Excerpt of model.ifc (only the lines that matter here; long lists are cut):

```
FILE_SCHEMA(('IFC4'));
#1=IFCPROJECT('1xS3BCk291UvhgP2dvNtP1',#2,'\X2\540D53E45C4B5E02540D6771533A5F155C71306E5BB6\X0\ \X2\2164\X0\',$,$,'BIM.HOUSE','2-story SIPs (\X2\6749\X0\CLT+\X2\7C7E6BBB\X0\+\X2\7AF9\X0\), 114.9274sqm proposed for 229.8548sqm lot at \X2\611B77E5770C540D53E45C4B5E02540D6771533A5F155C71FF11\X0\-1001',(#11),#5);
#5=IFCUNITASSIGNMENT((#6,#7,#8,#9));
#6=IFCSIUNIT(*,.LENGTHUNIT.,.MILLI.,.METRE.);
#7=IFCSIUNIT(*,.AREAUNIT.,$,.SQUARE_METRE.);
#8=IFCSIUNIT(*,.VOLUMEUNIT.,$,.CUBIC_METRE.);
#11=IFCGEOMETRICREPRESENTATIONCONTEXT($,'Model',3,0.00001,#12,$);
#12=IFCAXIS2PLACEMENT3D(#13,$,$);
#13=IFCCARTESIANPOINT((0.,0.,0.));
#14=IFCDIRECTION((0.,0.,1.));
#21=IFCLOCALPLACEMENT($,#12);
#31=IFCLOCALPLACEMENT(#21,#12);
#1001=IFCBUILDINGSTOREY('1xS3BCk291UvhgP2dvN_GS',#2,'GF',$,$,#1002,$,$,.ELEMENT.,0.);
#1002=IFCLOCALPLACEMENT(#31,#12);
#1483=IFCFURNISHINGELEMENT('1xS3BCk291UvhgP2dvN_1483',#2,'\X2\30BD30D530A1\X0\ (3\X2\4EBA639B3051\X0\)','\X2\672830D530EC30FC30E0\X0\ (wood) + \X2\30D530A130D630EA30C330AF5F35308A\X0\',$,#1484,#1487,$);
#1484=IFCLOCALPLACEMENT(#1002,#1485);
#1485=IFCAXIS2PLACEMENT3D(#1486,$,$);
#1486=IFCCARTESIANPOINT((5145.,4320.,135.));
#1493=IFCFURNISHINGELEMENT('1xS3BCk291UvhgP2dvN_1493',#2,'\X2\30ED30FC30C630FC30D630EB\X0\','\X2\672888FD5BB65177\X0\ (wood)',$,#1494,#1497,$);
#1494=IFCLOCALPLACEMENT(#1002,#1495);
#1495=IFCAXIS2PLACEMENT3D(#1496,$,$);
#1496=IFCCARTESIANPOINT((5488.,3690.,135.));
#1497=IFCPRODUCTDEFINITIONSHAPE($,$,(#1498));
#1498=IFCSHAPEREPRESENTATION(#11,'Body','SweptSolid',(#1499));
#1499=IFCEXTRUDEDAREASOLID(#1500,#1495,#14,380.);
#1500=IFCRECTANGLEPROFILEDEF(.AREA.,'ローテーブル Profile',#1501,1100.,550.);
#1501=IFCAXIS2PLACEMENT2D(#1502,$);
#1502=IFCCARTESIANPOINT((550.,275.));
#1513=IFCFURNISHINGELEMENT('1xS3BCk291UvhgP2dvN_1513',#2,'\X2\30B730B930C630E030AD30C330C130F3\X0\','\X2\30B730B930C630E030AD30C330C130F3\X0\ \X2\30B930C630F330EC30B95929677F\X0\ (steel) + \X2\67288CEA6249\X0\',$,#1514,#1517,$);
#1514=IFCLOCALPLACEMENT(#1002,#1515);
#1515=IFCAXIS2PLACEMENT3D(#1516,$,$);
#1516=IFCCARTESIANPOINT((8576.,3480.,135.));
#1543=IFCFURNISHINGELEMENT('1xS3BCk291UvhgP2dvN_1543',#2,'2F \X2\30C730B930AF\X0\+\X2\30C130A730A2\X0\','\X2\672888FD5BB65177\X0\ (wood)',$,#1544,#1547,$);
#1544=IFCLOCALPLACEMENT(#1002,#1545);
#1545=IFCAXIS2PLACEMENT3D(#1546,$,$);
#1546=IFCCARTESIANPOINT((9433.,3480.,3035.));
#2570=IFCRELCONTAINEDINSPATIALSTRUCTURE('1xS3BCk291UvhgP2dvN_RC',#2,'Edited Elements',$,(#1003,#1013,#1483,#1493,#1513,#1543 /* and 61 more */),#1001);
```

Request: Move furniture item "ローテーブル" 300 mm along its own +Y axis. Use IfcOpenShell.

```python
import ifcopenshell
import ifcopenshell.api.geometry
import ifcopenshell.util.placement

model = ifcopenshell.open("model.ifc")

item = model.by_id(1493)
matrix = ifcopenshell.util.placement.get_local_placement(item.ObjectPlacement)
matrix[:3, 3] += matrix[:3, 1] * 300.0
ifcopenshell.api.geometry.edit_object_placement(model, product=item, matrix=matrix, is_si=False)

print(ifcopenshell.util.placement.get_local_placement(item.ObjectPlacement).round(3) + 0.0)

model.write("model_v2.ifc")
```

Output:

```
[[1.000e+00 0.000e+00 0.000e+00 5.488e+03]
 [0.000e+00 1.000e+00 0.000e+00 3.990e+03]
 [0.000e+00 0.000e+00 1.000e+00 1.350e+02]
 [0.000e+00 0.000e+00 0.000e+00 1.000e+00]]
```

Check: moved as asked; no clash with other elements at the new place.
